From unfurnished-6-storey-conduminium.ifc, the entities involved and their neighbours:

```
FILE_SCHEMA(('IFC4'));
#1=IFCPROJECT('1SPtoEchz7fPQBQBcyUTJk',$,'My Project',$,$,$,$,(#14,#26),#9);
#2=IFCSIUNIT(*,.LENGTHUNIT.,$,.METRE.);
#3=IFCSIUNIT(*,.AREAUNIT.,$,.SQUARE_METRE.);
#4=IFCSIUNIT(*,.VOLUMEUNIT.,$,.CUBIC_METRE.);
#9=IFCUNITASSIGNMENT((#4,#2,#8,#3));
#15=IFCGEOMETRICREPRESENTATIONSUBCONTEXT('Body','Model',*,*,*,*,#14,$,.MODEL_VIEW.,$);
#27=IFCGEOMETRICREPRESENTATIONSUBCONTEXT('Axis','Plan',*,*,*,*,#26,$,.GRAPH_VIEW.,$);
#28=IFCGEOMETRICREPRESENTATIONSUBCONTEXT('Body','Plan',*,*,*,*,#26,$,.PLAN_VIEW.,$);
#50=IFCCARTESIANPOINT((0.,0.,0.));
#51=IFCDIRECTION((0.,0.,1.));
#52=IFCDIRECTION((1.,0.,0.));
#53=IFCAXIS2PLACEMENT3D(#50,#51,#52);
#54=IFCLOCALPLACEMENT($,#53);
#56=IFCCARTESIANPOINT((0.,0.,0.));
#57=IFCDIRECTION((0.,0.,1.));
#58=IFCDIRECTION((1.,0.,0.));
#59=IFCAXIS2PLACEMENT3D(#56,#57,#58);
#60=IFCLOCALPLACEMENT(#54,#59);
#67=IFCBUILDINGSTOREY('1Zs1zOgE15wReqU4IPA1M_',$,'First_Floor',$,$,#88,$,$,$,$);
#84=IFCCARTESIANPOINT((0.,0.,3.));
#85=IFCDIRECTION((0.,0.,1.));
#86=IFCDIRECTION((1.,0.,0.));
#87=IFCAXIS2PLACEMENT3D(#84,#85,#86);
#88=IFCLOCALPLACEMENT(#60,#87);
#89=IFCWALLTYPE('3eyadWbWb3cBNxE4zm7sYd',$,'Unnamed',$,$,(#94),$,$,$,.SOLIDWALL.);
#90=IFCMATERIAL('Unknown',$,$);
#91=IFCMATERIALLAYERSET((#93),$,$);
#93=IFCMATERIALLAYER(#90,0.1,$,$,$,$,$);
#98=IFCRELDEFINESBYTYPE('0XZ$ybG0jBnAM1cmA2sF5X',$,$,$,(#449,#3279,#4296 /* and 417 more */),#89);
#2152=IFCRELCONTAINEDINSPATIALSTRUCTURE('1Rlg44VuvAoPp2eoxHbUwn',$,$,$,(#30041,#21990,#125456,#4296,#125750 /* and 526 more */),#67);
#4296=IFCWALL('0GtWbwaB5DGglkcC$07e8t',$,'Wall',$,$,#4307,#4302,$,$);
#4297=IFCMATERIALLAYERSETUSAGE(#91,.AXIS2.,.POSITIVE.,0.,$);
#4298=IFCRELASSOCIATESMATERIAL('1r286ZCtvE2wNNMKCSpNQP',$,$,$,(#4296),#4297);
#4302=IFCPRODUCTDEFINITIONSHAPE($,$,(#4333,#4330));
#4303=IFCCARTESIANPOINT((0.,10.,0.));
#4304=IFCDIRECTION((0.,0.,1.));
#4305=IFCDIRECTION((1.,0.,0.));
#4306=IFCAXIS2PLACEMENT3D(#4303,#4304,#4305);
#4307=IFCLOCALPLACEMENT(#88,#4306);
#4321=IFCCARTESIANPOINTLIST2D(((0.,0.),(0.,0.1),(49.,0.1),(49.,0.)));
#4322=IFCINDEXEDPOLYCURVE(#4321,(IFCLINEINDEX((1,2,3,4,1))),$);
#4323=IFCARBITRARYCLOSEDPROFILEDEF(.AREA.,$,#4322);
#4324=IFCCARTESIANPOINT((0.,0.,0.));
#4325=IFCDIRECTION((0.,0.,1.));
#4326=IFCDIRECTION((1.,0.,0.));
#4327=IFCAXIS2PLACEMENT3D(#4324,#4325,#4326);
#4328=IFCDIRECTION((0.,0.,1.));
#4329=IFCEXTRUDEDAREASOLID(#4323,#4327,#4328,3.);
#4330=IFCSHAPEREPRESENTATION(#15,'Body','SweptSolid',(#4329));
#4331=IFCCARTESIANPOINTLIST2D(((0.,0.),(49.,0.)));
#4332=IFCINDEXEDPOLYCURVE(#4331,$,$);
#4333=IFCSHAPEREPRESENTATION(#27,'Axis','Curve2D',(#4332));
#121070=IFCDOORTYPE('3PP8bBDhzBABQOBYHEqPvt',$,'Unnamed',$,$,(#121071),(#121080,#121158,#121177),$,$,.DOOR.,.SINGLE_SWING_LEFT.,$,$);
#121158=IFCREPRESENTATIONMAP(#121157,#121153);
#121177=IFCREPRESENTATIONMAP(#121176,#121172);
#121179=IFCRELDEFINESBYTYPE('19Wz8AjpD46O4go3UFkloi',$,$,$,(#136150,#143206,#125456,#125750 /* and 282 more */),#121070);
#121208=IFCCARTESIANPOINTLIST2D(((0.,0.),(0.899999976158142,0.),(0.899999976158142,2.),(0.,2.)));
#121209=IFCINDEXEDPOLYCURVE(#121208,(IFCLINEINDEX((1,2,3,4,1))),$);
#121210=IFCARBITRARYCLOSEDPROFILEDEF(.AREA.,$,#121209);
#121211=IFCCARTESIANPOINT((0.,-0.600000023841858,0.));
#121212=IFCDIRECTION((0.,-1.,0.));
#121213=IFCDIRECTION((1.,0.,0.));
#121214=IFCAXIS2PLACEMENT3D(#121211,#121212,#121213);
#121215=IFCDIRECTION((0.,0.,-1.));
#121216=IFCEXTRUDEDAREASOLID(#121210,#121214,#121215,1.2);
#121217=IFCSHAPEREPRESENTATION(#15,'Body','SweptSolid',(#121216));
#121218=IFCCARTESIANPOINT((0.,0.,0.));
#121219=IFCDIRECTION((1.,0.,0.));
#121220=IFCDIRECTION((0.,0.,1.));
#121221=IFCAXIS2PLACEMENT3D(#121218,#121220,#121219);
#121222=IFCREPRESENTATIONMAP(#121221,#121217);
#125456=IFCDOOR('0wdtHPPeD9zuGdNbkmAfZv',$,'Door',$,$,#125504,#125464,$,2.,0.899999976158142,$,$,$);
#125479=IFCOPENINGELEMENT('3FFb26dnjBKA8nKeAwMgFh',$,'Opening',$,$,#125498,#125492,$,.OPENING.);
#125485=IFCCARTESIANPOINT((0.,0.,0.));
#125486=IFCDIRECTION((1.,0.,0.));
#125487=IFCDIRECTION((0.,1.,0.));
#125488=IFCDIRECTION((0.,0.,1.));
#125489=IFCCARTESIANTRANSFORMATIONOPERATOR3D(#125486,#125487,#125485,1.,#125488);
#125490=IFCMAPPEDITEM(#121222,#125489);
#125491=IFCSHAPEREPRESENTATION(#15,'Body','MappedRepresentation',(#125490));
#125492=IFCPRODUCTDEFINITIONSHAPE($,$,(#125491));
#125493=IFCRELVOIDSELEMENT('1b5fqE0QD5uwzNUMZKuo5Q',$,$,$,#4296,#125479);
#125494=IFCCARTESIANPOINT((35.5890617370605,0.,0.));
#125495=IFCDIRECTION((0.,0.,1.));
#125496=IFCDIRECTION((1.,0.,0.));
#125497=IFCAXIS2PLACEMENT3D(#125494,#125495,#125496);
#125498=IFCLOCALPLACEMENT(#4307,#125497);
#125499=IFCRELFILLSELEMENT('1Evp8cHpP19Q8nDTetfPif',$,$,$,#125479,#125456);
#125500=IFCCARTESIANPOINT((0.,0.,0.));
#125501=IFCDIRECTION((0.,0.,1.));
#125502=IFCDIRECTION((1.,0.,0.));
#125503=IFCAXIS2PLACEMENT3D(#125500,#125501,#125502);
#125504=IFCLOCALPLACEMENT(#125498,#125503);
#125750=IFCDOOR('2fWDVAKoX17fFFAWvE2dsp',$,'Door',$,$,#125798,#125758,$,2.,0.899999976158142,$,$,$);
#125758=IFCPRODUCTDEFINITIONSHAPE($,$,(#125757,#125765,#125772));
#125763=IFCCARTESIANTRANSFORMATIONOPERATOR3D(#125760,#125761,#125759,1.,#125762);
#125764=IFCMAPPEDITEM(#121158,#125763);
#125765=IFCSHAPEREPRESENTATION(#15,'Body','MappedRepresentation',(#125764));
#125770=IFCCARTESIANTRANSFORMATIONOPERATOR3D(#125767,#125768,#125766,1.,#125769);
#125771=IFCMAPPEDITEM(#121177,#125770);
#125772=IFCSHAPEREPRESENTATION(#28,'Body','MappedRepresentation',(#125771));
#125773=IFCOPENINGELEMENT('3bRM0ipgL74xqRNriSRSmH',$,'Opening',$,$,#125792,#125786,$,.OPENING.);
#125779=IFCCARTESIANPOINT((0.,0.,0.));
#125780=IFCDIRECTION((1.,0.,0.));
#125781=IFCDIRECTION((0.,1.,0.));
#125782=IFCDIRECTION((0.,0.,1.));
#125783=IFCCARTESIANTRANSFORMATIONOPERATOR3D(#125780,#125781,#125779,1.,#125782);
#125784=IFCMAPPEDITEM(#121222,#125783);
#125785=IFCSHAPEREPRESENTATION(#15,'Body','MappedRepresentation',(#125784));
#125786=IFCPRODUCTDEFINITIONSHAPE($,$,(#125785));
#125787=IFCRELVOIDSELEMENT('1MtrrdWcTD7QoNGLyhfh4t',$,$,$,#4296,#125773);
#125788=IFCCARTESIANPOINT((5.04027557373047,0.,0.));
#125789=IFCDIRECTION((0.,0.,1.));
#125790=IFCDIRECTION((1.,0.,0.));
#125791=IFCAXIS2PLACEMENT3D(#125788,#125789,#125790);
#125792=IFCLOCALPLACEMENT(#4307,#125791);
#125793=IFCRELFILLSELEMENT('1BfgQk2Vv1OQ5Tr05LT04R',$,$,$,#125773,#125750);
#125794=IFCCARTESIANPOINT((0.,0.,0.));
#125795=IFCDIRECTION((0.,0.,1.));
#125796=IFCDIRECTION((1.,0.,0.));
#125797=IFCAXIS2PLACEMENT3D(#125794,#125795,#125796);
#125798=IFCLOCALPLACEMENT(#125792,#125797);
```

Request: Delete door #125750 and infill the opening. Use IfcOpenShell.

```python
import ifcopenshell
import ifcopenshell.api.feature
import ifcopenshell.api.root
import ifcopenshell.geom
import ifcopenshell.util.shape

model = ifcopenshell.open("unfurnished-6-storey-conduminium.ifc")
settings = ifcopenshell.geom.settings()


def volume(element):
    """Net volume in cubic metres, openings subtracted."""
    shape = ifcopenshell.geom.create_shape(settings, element)
    return ifcopenshell.util.shape.get_volume(shape.geometry)


door = model.by_id(125750)
opening = door.FillsVoids[0].RelatingOpeningElement
wall = opening.VoidsElements[0].RelatingBuildingElement
before = volume(wall)

ifcopenshell.api.root.remove_product(model, product=door)
ifcopenshell.api.feature.remove_feature(model, feature=opening)

after = volume(wall)

print(f"wall volume {before:.3f} -> {after:.3f} m3")

model.write("unfurnished-6-storey-conduminium_updated.ifc")
```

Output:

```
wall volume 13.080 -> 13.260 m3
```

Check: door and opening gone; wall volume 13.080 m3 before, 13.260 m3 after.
